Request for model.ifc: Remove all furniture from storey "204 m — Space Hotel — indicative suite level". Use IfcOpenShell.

First a look at what the model holds.

```python
import ifcopenshell
import ifcopenshell.util.element

model = ifcopenshell.open("model.ifc")
print(model.schema)
storey = next(s for s in model.by_type("IfcBuildingStorey") if s.Name == "204 m — Space Hotel — indicative suite level")
furniture = [e for e in ifcopenshell.util.element.get_decomposition(storey) if e.is_a("IfcFurnishingElement")]
seen = {}
for e in furniture:
    element_type = ifcopenshell.util.element.get_type(e)
    name = element_type.Name if element_type not in (None, e) else None
    seen[name] = seen.get(name, 0) + 1
for name, count in sorted(seen.items(), key=str):
    print(count, "x", name)
```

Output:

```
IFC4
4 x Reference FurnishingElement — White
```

```python
import ifcopenshell
import ifcopenshell.api.root
import ifcopenshell.util.element

model = ifcopenshell.open("model.ifc")

storey = next(s for s in model.by_type("IfcBuildingStorey") if s.Name == "204 m — Space Hotel — indicative suite level")
furniture = [e for e in ifcopenshell.util.element.get_decomposition(storey) if e.is_a("IfcFurnishingElement")]

for e in furniture:
    ifcopenshell.api.root.remove_product(model, product=e)
print(len(furniture), "removed")

model.write("model_rev.ifc")
```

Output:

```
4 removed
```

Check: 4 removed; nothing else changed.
